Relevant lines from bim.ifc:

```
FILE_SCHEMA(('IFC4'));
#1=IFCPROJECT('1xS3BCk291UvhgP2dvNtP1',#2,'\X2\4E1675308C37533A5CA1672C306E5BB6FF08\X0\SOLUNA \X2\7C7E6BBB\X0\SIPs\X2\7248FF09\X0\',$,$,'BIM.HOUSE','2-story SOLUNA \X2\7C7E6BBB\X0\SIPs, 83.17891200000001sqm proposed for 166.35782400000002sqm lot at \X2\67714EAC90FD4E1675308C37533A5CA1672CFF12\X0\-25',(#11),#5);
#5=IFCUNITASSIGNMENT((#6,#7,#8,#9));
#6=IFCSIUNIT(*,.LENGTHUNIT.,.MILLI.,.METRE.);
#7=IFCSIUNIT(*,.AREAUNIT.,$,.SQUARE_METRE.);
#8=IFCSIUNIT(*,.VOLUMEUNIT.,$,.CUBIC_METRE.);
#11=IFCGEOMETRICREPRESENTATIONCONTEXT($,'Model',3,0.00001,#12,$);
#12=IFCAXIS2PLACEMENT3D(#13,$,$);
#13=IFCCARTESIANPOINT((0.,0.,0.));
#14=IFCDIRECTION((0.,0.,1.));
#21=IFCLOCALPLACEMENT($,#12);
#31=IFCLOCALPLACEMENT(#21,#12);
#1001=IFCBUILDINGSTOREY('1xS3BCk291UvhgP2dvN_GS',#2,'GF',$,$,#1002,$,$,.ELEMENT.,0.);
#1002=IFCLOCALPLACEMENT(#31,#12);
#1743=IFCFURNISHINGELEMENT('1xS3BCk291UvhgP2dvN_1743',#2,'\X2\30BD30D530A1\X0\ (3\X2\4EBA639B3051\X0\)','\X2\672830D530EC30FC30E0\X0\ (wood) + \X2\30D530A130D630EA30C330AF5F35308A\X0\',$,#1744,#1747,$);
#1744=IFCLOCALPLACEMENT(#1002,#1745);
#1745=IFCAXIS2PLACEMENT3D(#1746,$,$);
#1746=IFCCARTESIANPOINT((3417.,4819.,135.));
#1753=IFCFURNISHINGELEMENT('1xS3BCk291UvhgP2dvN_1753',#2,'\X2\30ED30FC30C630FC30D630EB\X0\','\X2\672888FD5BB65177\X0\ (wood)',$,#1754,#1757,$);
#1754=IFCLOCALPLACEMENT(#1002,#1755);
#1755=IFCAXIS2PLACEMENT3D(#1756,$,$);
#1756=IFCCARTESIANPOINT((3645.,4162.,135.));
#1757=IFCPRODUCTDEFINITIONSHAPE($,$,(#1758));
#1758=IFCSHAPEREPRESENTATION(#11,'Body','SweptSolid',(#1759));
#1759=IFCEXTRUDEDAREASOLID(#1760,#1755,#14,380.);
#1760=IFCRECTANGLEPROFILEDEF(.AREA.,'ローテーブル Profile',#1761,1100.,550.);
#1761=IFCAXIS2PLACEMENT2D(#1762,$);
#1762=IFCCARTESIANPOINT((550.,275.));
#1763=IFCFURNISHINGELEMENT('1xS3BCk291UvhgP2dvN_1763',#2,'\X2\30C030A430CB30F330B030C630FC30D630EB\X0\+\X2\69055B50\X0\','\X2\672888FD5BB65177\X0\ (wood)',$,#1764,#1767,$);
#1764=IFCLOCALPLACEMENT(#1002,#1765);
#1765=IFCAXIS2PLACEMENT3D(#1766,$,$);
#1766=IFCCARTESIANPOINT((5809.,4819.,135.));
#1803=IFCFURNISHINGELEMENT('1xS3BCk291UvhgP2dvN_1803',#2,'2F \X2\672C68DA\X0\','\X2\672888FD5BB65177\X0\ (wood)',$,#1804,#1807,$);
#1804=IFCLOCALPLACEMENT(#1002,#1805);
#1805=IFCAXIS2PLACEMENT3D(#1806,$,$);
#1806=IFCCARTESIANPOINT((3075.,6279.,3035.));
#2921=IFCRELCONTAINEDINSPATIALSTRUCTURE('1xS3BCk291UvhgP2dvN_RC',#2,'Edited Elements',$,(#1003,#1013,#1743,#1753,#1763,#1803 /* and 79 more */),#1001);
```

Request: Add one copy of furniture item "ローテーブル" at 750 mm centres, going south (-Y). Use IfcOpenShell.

```python
import numpy as np
import ifcopenshell
import ifcopenshell.api.geometry
import ifcopenshell.api.root
import ifcopenshell.util.element
import ifcopenshell.util.placement

model = ifcopenshell.open("bim.ifc")


def reuse_history(source, copy):
    """copy_class also copies each property set's owner history, people and application; keep the originals."""
    for rel in copy.IsDefinedBy:
        if rel.is_a("IfcRelDefinesByProperties") and (history := rel.RelatingPropertyDefinition.OwnerHistory):
            rel.RelatingPropertyDefinition.OwnerHistory = source.OwnerHistory
            ifcopenshell.util.element.remove_deep2(model, history)


source = model.by_id(1753)
base = ifcopenshell.util.placement.get_local_placement(source.ObjectPlacement)
step = np.array([0.0, -1.0, 0.0]) * 750.0

for i in range(1, 2):
    copy = ifcopenshell.api.root.copy_class(model, product=source)
    copy.Representation = ifcopenshell.util.element.copy_deep(
        model, source.Representation, exclude=["IfcGeometricRepresentationContext", "IfcRepresentationMap"]
    )
    reuse_history(source, copy)
    matrix = base.copy()
    matrix[:3, 3] += i * step
    print("added at", matrix[:3, 3].round(3) + 0.0)
    ifcopenshell.api.geometry.edit_object_placement(model, product=copy, matrix=matrix, is_si=False)

model.write("bim_updated.ifc")
```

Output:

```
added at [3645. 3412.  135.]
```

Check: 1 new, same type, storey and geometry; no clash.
